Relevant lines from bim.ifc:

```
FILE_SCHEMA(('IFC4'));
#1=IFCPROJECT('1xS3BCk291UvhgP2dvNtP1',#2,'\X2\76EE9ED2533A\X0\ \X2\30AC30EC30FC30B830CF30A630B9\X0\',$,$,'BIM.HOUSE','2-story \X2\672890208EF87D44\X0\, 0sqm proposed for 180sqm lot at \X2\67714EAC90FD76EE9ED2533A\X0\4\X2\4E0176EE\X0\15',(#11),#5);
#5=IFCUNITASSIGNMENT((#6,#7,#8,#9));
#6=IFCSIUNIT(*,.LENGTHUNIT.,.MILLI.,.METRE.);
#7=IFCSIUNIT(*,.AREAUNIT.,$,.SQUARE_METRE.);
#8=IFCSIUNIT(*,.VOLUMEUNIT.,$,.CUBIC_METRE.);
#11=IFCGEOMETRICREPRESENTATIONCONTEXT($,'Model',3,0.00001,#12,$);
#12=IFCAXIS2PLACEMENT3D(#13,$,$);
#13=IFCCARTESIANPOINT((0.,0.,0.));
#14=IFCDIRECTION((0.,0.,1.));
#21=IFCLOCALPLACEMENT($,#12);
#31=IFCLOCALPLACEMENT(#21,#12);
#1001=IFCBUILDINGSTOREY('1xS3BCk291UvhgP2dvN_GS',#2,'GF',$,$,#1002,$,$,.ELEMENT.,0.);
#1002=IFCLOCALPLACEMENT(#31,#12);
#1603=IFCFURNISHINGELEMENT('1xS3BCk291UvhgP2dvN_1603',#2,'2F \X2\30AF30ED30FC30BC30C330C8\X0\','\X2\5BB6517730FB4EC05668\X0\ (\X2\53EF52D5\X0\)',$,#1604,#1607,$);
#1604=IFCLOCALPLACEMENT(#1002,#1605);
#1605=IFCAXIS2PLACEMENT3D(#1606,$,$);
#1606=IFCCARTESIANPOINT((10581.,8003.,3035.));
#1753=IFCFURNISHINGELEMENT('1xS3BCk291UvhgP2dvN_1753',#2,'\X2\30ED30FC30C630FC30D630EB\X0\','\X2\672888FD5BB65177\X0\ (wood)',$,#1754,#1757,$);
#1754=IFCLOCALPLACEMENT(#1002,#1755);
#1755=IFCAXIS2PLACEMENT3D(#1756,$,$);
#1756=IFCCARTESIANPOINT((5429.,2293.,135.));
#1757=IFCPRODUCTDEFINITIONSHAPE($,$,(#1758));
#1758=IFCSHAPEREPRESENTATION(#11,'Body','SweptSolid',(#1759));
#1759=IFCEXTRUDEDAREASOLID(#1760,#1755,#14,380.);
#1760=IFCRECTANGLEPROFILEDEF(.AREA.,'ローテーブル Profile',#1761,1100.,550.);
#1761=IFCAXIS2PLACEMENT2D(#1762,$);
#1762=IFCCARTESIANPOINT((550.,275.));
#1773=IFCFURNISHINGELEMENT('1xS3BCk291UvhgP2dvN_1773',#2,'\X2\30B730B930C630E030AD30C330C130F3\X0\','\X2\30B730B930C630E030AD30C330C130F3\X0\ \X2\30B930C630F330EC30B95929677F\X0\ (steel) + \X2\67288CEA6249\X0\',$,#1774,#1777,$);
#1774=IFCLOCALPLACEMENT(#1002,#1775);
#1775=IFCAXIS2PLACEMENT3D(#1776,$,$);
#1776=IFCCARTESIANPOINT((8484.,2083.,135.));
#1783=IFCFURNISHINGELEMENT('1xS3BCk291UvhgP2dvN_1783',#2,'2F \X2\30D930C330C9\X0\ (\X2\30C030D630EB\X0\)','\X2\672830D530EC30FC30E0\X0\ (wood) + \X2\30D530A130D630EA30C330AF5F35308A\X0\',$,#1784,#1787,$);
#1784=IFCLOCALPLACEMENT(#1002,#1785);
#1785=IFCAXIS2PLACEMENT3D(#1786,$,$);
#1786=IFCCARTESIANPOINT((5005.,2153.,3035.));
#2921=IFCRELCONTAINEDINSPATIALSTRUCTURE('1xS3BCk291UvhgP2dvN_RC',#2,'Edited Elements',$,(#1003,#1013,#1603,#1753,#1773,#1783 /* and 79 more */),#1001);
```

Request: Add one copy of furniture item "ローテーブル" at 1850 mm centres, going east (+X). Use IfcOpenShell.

```python
import numpy as np
import ifcopenshell
import ifcopenshell.api.geometry
import ifcopenshell.api.root
import ifcopenshell.util.element
import ifcopenshell.util.placement

model = ifcopenshell.open("bim.ifc")


def reuse_history(source, copy):
    """copy_class also copies each property set's owner history, people and application; keep the originals."""
    for rel in copy.IsDefinedBy:
        if rel.is_a("IfcRelDefinesByProperties") and (history := rel.RelatingPropertyDefinition.OwnerHistory):
            rel.RelatingPropertyDefinition.OwnerHistory = source.OwnerHistory
            ifcopenshell.util.element.remove_deep2(model, history)


source = model.by_id(1753)
base = ifcopenshell.util.placement.get_local_placement(source.ObjectPlacement)
step = np.array([1.0, 0.0, 0.0]) * 1850.0

for i in range(1, 2):
    copy = ifcopenshell.api.root.copy_class(model, product=source)
    copy.Representation = ifcopenshell.util.element.copy_deep(
        model, source.Representation, exclude=["IfcGeometricRepresentationContext", "IfcRepresentationMap"]
    )
    reuse_history(source, copy)
    matrix = base.copy()
    matrix[:3, 3] += i * step
    print("added at", matrix[:3, 3].round(3) + 0.0)
    ifcopenshell.api.geometry.edit_object_placement(model, product=copy, matrix=matrix, is_si=False)

model.write("bim_rev.ifc")
```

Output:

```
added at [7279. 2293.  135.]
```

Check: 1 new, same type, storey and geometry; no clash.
